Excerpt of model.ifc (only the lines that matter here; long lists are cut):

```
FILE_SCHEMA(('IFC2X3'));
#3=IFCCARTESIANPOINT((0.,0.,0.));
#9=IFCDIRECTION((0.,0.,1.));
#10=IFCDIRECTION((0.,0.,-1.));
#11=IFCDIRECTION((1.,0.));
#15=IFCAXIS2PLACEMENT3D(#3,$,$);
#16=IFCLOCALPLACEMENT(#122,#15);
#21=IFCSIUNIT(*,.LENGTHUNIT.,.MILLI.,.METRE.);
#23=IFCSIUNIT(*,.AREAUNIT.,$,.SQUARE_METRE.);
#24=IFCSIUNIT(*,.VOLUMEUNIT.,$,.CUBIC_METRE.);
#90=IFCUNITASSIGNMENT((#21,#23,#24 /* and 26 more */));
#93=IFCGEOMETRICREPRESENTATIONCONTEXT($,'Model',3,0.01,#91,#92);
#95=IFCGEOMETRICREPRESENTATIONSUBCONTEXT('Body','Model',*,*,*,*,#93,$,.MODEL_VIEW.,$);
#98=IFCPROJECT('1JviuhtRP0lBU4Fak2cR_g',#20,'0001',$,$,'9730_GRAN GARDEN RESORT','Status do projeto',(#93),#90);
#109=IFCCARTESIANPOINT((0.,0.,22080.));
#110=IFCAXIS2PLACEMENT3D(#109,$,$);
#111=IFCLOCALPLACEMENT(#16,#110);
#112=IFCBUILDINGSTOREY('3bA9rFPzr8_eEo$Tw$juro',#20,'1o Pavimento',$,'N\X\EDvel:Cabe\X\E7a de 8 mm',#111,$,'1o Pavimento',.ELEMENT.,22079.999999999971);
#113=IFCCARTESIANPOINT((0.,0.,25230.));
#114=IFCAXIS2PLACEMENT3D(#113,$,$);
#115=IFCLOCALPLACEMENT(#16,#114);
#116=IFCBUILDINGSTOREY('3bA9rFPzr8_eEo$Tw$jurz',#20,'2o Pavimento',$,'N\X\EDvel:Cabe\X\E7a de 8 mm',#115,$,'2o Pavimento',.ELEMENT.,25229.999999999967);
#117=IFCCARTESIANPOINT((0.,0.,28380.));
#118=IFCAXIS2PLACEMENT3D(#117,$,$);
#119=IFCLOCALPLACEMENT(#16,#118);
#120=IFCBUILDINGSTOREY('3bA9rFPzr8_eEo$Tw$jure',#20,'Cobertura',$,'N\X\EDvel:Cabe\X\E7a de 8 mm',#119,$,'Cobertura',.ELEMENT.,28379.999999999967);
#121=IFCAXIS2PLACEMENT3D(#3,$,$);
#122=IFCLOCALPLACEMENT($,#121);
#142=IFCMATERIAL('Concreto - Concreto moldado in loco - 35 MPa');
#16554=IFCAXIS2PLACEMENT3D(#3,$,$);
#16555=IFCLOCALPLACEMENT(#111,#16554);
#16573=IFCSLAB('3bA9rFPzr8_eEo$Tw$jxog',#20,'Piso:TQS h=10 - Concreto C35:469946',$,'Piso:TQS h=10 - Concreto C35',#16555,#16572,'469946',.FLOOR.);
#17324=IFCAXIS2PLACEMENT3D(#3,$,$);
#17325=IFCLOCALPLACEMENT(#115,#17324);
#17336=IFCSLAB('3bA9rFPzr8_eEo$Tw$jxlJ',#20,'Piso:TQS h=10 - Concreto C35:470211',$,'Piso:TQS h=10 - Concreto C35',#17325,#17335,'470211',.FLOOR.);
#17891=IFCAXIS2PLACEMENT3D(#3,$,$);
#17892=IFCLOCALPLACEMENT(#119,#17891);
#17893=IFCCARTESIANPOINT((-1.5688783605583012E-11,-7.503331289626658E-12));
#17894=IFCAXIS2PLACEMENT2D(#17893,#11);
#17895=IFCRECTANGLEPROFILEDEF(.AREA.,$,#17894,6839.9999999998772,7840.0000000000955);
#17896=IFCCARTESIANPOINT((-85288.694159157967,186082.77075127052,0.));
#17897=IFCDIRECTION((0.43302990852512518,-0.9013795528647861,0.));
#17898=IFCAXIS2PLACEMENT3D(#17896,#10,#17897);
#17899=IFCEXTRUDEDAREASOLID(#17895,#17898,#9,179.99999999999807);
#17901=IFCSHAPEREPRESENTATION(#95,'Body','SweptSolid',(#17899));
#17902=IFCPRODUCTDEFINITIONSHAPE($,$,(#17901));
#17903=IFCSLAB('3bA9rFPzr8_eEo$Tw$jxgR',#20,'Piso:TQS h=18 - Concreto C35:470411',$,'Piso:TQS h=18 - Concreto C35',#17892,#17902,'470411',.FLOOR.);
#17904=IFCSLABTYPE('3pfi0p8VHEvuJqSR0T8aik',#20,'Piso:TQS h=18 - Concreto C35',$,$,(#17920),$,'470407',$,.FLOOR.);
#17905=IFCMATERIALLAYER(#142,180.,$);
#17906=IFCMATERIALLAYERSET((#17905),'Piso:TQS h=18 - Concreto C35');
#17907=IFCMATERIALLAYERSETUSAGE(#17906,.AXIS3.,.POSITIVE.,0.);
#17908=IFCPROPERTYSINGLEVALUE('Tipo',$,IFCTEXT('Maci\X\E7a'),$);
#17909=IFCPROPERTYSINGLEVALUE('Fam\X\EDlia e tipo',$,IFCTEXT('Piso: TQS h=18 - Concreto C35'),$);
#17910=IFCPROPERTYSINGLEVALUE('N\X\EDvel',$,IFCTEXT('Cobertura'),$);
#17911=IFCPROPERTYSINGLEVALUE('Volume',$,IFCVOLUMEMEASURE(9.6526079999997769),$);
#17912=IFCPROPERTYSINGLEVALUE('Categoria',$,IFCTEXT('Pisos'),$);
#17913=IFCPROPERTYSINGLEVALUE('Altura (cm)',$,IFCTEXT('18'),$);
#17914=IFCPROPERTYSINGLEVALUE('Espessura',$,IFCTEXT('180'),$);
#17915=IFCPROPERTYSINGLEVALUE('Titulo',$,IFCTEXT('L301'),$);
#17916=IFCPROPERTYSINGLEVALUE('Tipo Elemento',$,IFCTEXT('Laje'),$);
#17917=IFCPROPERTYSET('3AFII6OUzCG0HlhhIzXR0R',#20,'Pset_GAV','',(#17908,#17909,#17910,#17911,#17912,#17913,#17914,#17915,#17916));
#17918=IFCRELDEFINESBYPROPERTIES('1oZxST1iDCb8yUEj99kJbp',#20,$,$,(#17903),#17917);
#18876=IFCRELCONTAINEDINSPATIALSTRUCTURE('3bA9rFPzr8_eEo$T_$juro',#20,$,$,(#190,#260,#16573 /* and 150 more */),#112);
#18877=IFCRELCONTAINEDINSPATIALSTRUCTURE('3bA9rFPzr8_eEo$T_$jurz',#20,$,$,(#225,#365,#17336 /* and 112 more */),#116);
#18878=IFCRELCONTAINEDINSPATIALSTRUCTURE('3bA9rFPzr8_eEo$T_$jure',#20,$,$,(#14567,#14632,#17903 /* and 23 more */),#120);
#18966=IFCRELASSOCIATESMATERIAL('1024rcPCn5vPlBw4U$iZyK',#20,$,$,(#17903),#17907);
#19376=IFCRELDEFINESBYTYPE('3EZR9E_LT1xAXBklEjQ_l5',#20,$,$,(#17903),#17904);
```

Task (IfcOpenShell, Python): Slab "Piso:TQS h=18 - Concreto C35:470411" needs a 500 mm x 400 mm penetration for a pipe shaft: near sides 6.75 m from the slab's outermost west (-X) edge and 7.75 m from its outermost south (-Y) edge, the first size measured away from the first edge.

```python
import numpy as np
import ifcopenshell
import ifcopenshell.api.feature
import ifcopenshell.api.geometry
import ifcopenshell.api.pset
import ifcopenshell.api.root
import ifcopenshell.geom
import ifcopenshell.util.element
import ifcopenshell.util.placement
import ifcopenshell.util.representation
import ifcopenshell.util.shape
import ifcopenshell.util.unit

model = ifcopenshell.open("model.ifc")
unit_scale = ifcopenshell.util.unit.calculate_unit_scale(model)
volume_scale = ifcopenshell.util.unit.calculate_unit_scale(model, "VOLUMEUNIT")
settings = ifcopenshell.geom.settings()


def volume(element):
    """Net volume in cubic metres, openings subtracted."""
    shape = ifcopenshell.geom.create_shape(settings, element)
    return ifcopenshell.util.shape.get_volume(shape.geometry)


slab = model.by_id(17903)
before = volume(slab)

# Extent in the slab's own axes, in metres. The edges named are its -X and -Y sides.
slab_shape = ifcopenshell.geom.create_shape(settings, slab)
vertices = ifcopenshell.util.shape.get_vertices(slab_shape.geometry)
x_min, y_min, bottom = vertices.min(axis=0)
top = vertices[:, 2].max()

opening = ifcopenshell.api.root.create_entity(model, ifc_class="IfcOpeningElement", name="Pipe shaft opening")
context = ifcopenshell.util.representation.get_context(model, "Model", "Body", "MODEL_VIEW")
width, depth = 0.5, 0.4
outline = [(0.0, 0.0), (width, 0.0), (width, depth), (0.0, depth), (0.0, 0.0)]
# Overshoot both faces by 50 mm so the cut is clean.
shape = ifcopenshell.api.geometry.add_slab_representation(
    model, context=context, depth=top - bottom + 0.1, polyline=outline
)
ifcopenshell.api.geometry.assign_representation(model, product=opening, representation=shape)

matrix = ifcopenshell.util.placement.get_local_placement(slab.ObjectPlacement)
matrix[:, 3] = matrix @ np.append(np.array([x_min + 6.75, y_min + 7.75, bottom - 0.05]) / unit_scale, 1.0)
ifcopenshell.api.geometry.edit_object_placement(model, product=opening, matrix=matrix, is_si=False)
ifcopenshell.api.feature.add_feature(model, feature=opening, element=slab)

after = volume(slab)

# Update the slab's stored quantities.
pset = model.by_id(ifcopenshell.util.element.get_pset(slab, "Pset_GAV", should_inherit=False)["id"])
ifcopenshell.api.pset.edit_pset(model, pset=pset, properties={
    "Volume": model.create_entity("IfcVolumeMeasure", after / volume_scale),
})

print(f"slab volume {before:.3f} -> {after:.3f} m3")

model.write("model_edited.ifc")
```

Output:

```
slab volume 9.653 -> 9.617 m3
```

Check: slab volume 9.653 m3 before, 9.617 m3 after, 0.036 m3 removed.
